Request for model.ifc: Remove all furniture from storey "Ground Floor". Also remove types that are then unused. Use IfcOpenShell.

First a look at what the model holds.

```python
import ifcopenshell
import ifcopenshell.util.element

model = ifcopenshell.open("model.ifc")
print(model.schema)
storey = next(s for s in model.by_type("IfcBuildingStorey") if s.Name == "Ground Floor")
furniture = [e for e in ifcopenshell.util.element.get_decomposition(storey) if e.is_a("IfcFurnishingElement")]
seen = {}
for e in furniture:
    element_type = ifcopenshell.util.element.get_type(e)
    name = element_type.Name if element_type not in (None, e) else None
    seen[name] = seen.get(name, 0) + 1
for name, count in sorted(seen.items(), key=str):
    print(count, "x", name)
```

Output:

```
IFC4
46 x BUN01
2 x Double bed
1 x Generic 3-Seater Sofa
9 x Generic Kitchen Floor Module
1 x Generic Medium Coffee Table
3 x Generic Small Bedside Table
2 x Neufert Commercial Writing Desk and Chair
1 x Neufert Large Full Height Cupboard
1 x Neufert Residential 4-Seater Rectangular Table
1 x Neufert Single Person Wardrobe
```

```python
import ifcopenshell
import ifcopenshell.api.root
import ifcopenshell.util.element

model = ifcopenshell.open("model.ifc")

storey = next(s for s in model.by_type("IfcBuildingStorey") if s.Name == "Ground Floor")
furniture = [e for e in ifcopenshell.util.element.get_decomposition(storey) if e.is_a("IfcFurnishingElement")]
types = {ifcopenshell.util.element.get_type(e) for e in furniture} - {None, *furniture}

for e in furniture:
    ifcopenshell.api.root.remove_product(model, product=e)
print(len(furniture), "removed")

unused = [t for t in types if not ifcopenshell.util.element.get_types(t)]
for t in unused:
    ifcopenshell.api.root.remove_product(model, product=t)
print(len(unused), "unused types removed")

model.write("model-out.ifc")
```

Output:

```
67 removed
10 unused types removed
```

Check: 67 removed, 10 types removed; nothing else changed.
